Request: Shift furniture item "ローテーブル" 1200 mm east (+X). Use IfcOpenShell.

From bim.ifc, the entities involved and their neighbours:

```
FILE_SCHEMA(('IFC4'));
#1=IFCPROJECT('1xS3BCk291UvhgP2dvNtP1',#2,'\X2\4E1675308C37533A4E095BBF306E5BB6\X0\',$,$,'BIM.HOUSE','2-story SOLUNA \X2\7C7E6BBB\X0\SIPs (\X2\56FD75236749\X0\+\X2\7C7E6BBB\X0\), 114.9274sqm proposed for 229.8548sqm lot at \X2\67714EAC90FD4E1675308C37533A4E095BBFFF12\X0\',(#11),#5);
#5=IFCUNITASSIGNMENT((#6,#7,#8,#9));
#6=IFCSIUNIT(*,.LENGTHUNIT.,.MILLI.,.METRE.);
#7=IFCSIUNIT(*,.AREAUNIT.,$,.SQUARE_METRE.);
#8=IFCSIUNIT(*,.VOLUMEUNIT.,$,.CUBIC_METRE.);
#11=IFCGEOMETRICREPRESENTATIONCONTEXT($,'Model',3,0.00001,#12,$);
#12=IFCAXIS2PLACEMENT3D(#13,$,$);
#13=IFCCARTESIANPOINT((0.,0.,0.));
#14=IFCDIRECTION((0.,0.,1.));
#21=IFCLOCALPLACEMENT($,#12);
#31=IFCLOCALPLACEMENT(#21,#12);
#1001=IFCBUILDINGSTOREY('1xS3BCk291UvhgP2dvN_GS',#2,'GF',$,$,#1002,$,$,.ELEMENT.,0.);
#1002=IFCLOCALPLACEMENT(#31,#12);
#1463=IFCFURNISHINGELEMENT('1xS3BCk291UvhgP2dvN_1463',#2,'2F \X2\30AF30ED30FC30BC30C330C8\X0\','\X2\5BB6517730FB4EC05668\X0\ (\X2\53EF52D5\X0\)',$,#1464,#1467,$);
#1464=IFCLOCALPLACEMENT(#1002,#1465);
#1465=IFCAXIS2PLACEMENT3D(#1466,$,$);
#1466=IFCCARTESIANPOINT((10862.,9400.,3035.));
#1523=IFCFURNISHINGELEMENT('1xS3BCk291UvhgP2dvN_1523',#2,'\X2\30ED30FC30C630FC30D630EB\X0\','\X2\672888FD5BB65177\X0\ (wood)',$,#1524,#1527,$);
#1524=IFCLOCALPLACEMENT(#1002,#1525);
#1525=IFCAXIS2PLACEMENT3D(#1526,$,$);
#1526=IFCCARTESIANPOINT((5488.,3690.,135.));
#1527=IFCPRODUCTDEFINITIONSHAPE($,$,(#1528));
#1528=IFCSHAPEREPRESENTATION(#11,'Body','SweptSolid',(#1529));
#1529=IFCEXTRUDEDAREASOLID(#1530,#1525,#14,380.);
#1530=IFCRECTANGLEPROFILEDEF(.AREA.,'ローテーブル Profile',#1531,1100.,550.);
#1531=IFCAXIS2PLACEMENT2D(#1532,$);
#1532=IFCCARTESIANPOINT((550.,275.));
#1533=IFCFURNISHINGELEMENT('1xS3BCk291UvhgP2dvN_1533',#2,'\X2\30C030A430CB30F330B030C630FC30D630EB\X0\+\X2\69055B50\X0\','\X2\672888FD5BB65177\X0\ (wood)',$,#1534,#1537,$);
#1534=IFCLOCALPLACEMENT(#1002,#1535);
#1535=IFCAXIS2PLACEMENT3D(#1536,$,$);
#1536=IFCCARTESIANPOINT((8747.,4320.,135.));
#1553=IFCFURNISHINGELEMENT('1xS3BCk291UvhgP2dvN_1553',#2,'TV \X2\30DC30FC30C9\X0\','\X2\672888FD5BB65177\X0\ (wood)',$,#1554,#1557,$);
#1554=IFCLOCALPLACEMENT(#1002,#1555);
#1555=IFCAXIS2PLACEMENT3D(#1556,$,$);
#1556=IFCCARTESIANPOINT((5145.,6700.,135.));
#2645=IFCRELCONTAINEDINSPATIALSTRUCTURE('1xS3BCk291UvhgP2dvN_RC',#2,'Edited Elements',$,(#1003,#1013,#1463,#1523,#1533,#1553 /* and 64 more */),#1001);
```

```python
import ifcopenshell
import ifcopenshell.api.geometry
import ifcopenshell.util.placement
import ifcopenshell.util.unit

model = ifcopenshell.open("bim.ifc")
unit_scale = ifcopenshell.util.unit.calculate_unit_scale(model)

item = model.by_guid("1xS3BCk291UvhgP2dvN_1523")
matrix = ifcopenshell.util.placement.get_local_placement(item.ObjectPlacement)
matrix[0, 3] += 1.2 / unit_scale
ifcopenshell.api.geometry.edit_object_placement(model, product=item, matrix=matrix, is_si=False)

print(ifcopenshell.util.placement.get_local_placement(item.ObjectPlacement).round(3) + 0.0)

model.write("bim_rev.ifc")
```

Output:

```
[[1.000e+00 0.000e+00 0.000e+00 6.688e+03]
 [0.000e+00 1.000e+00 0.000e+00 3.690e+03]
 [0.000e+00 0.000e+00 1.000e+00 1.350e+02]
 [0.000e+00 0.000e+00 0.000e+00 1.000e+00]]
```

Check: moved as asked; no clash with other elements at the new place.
